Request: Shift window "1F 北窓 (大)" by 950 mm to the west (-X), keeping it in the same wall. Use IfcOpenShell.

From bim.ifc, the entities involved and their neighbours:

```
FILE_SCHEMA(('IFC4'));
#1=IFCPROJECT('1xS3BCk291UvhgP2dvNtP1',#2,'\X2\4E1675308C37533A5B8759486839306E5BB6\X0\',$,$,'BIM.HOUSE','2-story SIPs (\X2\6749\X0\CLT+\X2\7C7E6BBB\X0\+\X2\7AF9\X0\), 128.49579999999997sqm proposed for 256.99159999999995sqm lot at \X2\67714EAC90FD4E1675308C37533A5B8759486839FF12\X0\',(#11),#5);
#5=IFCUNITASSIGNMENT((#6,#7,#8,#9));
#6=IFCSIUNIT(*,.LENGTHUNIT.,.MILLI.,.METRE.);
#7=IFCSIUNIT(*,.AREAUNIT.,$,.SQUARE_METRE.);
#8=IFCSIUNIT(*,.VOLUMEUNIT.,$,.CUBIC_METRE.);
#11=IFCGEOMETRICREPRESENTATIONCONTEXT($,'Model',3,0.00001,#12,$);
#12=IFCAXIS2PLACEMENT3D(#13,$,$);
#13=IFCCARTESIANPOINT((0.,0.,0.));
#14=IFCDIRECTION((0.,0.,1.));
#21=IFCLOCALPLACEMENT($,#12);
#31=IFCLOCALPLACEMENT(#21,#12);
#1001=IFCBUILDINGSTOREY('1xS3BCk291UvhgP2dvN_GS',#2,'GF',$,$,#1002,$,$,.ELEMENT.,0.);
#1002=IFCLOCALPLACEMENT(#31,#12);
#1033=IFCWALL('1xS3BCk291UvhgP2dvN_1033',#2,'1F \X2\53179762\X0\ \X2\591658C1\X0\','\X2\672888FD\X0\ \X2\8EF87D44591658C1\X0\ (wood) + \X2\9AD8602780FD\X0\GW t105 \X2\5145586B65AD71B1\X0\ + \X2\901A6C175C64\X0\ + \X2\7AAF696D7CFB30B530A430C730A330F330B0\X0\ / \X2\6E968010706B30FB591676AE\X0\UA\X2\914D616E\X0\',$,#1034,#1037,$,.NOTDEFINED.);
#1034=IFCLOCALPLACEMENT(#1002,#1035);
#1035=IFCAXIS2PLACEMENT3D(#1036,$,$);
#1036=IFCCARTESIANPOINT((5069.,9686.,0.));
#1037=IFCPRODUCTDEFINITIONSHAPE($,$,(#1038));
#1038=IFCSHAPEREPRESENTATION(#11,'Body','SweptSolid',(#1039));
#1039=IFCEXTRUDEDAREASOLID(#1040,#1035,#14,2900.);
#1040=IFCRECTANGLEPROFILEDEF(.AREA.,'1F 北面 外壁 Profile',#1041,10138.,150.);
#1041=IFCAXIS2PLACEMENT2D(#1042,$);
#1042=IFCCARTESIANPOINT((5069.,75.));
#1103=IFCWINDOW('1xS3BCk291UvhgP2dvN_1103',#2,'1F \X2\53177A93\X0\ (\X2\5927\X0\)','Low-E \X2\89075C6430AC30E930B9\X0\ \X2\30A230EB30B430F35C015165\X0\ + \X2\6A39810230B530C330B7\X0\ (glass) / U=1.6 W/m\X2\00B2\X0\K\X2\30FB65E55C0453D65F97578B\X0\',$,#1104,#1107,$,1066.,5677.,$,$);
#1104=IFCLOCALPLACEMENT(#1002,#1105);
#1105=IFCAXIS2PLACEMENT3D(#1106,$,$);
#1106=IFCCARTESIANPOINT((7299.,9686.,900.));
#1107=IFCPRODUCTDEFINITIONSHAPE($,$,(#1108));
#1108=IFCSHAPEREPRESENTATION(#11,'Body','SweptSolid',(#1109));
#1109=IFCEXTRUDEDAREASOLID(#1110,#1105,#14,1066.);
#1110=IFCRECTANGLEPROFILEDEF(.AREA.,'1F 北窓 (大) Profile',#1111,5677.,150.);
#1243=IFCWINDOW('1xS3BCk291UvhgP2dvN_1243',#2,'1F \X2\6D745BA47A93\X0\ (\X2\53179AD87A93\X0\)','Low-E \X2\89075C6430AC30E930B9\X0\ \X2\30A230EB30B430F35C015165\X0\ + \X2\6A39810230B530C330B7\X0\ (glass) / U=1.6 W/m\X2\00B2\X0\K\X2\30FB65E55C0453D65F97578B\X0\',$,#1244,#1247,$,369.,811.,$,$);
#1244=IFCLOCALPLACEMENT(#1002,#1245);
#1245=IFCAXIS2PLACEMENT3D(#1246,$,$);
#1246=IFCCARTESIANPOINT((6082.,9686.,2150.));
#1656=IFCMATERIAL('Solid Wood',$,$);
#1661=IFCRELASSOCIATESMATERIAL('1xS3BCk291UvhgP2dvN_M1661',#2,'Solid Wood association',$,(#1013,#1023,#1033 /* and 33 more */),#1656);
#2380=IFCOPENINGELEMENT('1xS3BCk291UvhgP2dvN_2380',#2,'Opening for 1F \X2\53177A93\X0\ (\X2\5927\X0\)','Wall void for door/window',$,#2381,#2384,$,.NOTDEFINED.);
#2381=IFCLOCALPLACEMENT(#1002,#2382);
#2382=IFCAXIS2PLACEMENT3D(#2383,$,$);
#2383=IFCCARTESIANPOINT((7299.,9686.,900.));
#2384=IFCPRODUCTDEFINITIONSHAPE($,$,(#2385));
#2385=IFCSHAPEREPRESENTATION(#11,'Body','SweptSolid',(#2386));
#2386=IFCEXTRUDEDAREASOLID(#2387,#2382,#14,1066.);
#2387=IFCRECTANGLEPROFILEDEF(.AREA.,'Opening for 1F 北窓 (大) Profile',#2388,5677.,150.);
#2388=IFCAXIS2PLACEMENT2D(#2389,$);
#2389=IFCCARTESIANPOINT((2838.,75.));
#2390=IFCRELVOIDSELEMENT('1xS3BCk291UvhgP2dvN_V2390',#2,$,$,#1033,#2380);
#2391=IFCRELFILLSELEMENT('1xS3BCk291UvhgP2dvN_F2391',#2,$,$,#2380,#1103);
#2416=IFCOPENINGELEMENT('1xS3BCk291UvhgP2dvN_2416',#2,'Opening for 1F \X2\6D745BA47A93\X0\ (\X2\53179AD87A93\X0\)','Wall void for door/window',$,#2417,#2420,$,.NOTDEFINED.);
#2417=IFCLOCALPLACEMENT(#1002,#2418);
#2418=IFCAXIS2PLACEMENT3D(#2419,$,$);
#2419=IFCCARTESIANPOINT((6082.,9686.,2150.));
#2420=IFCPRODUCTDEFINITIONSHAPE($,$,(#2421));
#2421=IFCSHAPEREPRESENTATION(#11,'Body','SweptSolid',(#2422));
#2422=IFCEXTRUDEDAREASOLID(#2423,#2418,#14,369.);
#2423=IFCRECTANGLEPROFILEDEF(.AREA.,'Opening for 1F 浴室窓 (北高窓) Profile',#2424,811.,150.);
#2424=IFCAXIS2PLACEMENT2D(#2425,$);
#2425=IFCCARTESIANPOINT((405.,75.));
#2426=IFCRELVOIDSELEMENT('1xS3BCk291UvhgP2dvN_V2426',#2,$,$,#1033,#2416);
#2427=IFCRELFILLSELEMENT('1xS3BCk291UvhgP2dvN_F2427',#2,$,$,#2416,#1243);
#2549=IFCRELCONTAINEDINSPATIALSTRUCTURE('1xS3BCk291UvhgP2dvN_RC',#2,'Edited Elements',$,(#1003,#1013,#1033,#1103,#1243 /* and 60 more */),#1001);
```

```python
import ifcopenshell
import ifcopenshell.api.geometry
import ifcopenshell.util.placement

model = ifcopenshell.open("bim.ifc")

window = model.by_guid("1xS3BCk291UvhgP2dvN_1103")
opening = window.FillsVoids[0].RelatingOpeningElement
wall = opening.VoidsElements[0].RelatingBuildingElement

wall_matrix = ifcopenshell.util.placement.get_local_placement(wall.ObjectPlacement)
shift = wall_matrix[:3, 0] * -950.0
before = ifcopenshell.util.placement.get_local_placement(window.ObjectPlacement)[:3, 3].copy()

# The window is not placed relative to its opening, so move both.
for product in (opening, window):
    matrix = ifcopenshell.util.placement.get_local_placement(product.ObjectPlacement)
    matrix[:3, 3] += shift
    ifcopenshell.api.geometry.edit_object_placement(model, product=product, matrix=matrix, is_si=False)

after = ifcopenshell.util.placement.get_local_placement(window.ObjectPlacement)[:3, 3]
print("window moved by", (after - before).round(3) + 0.0)

model.write("bim_edited.ifc")
```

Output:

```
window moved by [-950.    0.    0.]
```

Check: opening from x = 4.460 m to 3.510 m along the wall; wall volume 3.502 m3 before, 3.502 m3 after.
